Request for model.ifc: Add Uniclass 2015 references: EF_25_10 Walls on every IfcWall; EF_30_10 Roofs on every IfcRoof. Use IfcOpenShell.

First a look at what the model holds.

```python
import ifcopenshell

model = ifcopenshell.open("model.ifc")
print(model.schema)
print("classifications:", [c.Name for c in model.by_type("IfcClassification")])
for ifc_class in ("IfcDoor", "IfcRoof", "IfcStair", "IfcWall", "IfcWindow"):
    print(ifc_class, len(model.by_type(ifc_class)))
```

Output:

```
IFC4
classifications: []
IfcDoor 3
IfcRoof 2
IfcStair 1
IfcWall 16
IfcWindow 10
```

```python
import ifcopenshell
import ifcopenshell.api.classification

model = ifcopenshell.open("model.ifc")

system = ifcopenshell.api.classification.add_classification(model, classification="Uniclass 2015")

codes = {
    "IfcWall": ("EF_25_10", "Walls"),
    "IfcRoof": ("EF_30_10", "Roofs"),
}
for ifc_class, (code, name) in codes.items():
    products = model.by_type(ifc_class)
    ifcopenshell.api.classification.add_reference(
        model, products=products, classification=system, identification=code, name=name
    )
    print(code, len(products))

model.write("model_edited.ifc")
```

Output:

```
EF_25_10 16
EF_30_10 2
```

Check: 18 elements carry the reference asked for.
